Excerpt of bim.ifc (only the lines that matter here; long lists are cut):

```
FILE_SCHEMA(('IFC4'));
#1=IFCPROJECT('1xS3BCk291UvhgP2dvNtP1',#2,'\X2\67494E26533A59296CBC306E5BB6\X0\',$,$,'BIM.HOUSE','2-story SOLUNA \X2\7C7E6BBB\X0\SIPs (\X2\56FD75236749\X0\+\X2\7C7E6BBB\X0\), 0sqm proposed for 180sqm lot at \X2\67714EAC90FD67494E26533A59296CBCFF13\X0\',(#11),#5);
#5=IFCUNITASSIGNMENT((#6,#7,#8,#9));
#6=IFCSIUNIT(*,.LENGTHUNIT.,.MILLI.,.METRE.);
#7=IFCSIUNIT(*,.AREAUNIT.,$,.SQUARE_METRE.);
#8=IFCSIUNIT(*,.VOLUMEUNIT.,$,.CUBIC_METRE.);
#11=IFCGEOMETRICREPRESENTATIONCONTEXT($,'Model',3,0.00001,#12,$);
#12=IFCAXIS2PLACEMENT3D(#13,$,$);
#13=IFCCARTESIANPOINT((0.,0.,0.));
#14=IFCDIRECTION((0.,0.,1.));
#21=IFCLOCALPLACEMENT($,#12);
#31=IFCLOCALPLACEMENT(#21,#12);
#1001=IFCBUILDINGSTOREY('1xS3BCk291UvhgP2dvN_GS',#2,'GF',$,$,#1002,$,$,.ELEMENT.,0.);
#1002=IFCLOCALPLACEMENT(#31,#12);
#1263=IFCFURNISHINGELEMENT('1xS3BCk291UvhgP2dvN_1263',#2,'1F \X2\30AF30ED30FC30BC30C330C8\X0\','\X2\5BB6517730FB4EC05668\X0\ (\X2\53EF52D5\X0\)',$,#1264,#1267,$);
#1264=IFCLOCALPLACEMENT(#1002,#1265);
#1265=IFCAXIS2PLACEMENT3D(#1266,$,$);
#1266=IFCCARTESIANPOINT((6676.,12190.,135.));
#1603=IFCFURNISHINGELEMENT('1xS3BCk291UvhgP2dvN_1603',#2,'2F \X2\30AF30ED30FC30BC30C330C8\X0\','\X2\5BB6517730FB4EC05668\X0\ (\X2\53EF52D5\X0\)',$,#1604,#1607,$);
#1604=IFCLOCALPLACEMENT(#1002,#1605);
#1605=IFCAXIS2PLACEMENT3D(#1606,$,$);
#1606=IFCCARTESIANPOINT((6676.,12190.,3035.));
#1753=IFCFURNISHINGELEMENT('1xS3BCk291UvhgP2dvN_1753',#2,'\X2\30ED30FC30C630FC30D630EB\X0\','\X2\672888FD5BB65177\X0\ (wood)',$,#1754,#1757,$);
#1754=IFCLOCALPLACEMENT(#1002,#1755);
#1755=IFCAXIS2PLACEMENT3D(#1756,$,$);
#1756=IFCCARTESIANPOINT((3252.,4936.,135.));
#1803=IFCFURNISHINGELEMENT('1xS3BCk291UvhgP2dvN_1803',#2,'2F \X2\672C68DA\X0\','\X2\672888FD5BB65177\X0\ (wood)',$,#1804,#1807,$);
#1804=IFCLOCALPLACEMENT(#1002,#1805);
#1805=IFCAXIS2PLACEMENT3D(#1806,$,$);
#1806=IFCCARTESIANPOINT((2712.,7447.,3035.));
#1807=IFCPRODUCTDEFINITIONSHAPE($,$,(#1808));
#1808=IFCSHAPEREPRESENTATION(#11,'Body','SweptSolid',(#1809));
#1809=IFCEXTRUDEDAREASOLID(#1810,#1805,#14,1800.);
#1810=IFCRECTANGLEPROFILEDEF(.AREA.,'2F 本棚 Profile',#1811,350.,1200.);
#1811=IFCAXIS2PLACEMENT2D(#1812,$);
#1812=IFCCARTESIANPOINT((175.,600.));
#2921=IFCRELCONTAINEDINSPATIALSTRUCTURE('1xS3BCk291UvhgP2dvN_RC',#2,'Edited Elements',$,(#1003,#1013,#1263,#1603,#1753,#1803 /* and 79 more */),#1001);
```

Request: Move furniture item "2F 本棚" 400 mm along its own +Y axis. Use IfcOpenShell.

```python
import ifcopenshell
import ifcopenshell.api.geometry
import ifcopenshell.util.placement

model = ifcopenshell.open("bim.ifc")

item = model.by_id(1803)
matrix = ifcopenshell.util.placement.get_local_placement(item.ObjectPlacement)
matrix[:3, 3] += matrix[:3, 1] * 400.0
ifcopenshell.api.geometry.edit_object_placement(model, product=item, matrix=matrix, is_si=False)

print(ifcopenshell.util.placement.get_local_placement(item.ObjectPlacement).round(3) + 0.0)

model.write("bim_updated.ifc")
```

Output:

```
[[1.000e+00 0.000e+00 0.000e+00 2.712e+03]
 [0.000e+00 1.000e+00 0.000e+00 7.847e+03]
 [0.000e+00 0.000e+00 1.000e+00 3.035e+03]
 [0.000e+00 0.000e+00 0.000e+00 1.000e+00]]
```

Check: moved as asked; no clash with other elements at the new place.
